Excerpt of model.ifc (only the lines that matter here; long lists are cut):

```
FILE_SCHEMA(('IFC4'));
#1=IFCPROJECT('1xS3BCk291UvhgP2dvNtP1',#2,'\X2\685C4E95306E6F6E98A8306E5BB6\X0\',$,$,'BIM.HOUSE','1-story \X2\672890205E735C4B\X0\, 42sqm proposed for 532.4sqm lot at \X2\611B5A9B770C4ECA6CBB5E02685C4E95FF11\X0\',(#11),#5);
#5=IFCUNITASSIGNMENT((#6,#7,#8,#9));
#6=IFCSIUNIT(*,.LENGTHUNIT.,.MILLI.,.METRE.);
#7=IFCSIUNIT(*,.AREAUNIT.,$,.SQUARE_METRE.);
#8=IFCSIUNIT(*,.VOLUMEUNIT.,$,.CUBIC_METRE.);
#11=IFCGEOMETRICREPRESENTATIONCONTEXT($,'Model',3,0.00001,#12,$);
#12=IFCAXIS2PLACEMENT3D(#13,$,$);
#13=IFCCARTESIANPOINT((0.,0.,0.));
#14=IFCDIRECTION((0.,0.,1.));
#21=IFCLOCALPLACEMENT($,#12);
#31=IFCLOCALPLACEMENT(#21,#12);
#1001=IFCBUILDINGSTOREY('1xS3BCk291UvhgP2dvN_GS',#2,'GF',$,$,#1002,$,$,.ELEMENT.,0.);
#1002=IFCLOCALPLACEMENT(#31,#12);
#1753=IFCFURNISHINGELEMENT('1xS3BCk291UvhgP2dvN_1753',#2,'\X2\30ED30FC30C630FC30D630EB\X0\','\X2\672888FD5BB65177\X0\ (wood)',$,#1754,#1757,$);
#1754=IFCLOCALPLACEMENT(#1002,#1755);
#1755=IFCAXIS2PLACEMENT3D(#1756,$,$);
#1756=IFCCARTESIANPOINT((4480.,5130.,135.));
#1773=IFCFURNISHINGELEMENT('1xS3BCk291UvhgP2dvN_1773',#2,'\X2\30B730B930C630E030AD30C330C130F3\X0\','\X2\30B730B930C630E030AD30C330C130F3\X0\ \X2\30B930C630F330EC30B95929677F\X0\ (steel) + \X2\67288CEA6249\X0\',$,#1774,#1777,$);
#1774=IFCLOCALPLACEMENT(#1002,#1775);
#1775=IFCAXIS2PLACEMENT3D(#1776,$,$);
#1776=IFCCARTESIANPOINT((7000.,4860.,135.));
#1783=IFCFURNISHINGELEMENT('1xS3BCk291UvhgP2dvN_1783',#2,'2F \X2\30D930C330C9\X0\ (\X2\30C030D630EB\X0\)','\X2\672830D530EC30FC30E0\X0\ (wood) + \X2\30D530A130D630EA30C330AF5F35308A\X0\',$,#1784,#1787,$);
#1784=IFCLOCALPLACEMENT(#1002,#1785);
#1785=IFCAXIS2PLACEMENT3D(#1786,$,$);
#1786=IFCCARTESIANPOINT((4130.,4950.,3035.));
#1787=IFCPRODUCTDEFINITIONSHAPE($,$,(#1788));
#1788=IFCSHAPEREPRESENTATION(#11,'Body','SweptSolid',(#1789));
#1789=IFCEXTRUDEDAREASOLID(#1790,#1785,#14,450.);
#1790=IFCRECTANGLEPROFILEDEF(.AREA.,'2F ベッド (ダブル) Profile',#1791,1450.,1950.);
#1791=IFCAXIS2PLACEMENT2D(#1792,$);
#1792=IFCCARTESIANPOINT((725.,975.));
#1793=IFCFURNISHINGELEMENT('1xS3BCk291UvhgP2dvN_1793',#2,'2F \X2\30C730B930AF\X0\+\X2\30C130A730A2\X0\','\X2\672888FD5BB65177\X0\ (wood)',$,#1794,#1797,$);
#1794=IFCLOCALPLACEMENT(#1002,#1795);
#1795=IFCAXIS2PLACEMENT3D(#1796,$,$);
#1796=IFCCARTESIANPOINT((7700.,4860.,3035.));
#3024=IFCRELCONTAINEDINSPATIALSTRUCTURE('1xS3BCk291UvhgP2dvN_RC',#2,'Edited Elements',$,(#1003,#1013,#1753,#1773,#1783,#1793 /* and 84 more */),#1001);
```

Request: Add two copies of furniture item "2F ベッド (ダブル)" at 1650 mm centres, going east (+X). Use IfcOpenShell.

```python
import numpy as np
import ifcopenshell
import ifcopenshell.api.geometry
import ifcopenshell.api.root
import ifcopenshell.util.element
import ifcopenshell.util.placement
import ifcopenshell.util.unit

model = ifcopenshell.open("model.ifc")
unit_scale = ifcopenshell.util.unit.calculate_unit_scale(model)


def reuse_history(source, copy):
    """copy_class also copies each property set's owner history, people and application; keep the originals."""
    for rel in copy.IsDefinedBy:
        if rel.is_a("IfcRelDefinesByProperties") and (history := rel.RelatingPropertyDefinition.OwnerHistory):
            rel.RelatingPropertyDefinition.OwnerHistory = source.OwnerHistory
            ifcopenshell.util.element.remove_deep2(model, history)


source = model.by_guid("1xS3BCk291UvhgP2dvN_1783")
base = ifcopenshell.util.placement.get_local_placement(source.ObjectPlacement)
step = np.array([1.0, 0.0, 0.0]) * 1.65 / unit_scale

for i in range(1, 3):
    copy = ifcopenshell.api.root.copy_class(model, product=source)
    copy.Representation = ifcopenshell.util.element.copy_deep(
        model, source.Representation, exclude=["IfcGeometricRepresentationContext", "IfcRepresentationMap"]
    )
    reuse_history(source, copy)
    matrix = base.copy()
    matrix[:3, 3] += i * step
    print("added at", matrix[:3, 3].round(3) + 0.0)
    ifcopenshell.api.geometry.edit_object_placement(model, product=copy, matrix=matrix, is_si=False)

model.write("model_updated.ifc")
```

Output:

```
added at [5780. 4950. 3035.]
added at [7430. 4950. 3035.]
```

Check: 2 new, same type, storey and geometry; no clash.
